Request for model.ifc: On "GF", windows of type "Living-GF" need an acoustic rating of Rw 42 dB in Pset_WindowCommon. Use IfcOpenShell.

First a look at what the model holds.

```python
import ifcopenshell
import ifcopenshell.util.element

model = ifcopenshell.open("model.ifc")
print(model.schema)
storey = next(s for s in model.by_type("IfcBuildingStorey") if s.Name == "GF")
windows = [e for e in ifcopenshell.util.element.get_decomposition(storey) if e.is_a("IfcWindow")]
seen = {}
for e in windows:
    element_type = ifcopenshell.util.element.get_type(e)
    key = (element_type.Name if element_type != e and element_type else None, ifcopenshell.util.element.get_pset(e, "Pset_WindowCommon", "AcousticRating"))
    seen[key] = seen.get(key, 0) + 1
for (name, value), count in sorted(seen.items(), key=str):
    print(count, "x", name, "|", value)
```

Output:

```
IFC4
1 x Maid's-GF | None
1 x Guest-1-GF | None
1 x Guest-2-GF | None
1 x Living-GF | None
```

```python
import ifcopenshell
import ifcopenshell.api.pset
import ifcopenshell.util.element

model = ifcopenshell.open("model.ifc")

storey = next(s for s in model.by_type("IfcBuildingStorey") if s.Name == "GF")
windows = [e for e in ifcopenshell.util.element.get_decomposition(storey) if e.is_a("IfcWindow")]

count = 0
for e in windows:
    element_type = ifcopenshell.util.element.get_type(e)
    if element_type in (None, e) or element_type.Name != "Living-GF":
        continue
    # add_pset returns the element's existing set when there is one.
    pset = ifcopenshell.api.pset.add_pset(model, product=e, name="Pset_WindowCommon")
    ifcopenshell.api.pset.edit_pset(model, pset=pset, properties={"AcousticRating": "Rw 42 dB"})
    count += 1

print(count, "windows updated")

model.write("model-out.ifc")
```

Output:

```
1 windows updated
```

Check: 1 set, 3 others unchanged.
